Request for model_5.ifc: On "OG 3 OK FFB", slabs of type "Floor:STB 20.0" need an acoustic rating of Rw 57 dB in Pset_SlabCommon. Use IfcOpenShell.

First a look at what the model holds.

```python
import ifcopenshell
import ifcopenshell.util.element

model = ifcopenshell.open("model_5.ifc")
print(model.schema)
storey = next(s for s in model.by_type("IfcBuildingStorey") if s.Name == "OG 3 OK FFB")
slabs = [e for e in ifcopenshell.util.element.get_decomposition(storey) if e.is_a("IfcSlab")]
seen = {}
for e in slabs:
    element_type = ifcopenshell.util.element.get_type(e)
    key = (element_type.Name if element_type != e and element_type else None, ifcopenshell.util.element.get_pset(e, "Pset_SlabCommon", "AcousticRating"))
    seen[key] = seen.get(key, 0) + 1
for (name, value), count in sorted(seen.items(), key=str):
    print(count, "x", name, "|", value)
```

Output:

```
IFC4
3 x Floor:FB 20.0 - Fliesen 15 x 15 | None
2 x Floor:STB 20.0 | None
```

```python
import ifcopenshell
import ifcopenshell.api.pset
import ifcopenshell.util.element

model = ifcopenshell.open("model_5.ifc")

storey = next(s for s in model.by_type("IfcBuildingStorey") if s.Name == "OG 3 OK FFB")
slabs = [e for e in ifcopenshell.util.element.get_decomposition(storey) if e.is_a("IfcSlab")]

count = 0
for e in slabs:
    element_type = ifcopenshell.util.element.get_type(e)
    if element_type in (None, e) or element_type.Name != "Floor:STB 20.0":
        continue
    # add_pset returns the element's existing set when there is one.
    pset = ifcopenshell.api.pset.add_pset(model, product=e, name="Pset_SlabCommon")
    ifcopenshell.api.pset.edit_pset(model, pset=pset, properties={"AcousticRating": "Rw 57 dB"})
    count += 1

print(count, "slabs updated")

model.write("model_5_updated.ifc")
```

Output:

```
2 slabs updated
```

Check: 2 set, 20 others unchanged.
